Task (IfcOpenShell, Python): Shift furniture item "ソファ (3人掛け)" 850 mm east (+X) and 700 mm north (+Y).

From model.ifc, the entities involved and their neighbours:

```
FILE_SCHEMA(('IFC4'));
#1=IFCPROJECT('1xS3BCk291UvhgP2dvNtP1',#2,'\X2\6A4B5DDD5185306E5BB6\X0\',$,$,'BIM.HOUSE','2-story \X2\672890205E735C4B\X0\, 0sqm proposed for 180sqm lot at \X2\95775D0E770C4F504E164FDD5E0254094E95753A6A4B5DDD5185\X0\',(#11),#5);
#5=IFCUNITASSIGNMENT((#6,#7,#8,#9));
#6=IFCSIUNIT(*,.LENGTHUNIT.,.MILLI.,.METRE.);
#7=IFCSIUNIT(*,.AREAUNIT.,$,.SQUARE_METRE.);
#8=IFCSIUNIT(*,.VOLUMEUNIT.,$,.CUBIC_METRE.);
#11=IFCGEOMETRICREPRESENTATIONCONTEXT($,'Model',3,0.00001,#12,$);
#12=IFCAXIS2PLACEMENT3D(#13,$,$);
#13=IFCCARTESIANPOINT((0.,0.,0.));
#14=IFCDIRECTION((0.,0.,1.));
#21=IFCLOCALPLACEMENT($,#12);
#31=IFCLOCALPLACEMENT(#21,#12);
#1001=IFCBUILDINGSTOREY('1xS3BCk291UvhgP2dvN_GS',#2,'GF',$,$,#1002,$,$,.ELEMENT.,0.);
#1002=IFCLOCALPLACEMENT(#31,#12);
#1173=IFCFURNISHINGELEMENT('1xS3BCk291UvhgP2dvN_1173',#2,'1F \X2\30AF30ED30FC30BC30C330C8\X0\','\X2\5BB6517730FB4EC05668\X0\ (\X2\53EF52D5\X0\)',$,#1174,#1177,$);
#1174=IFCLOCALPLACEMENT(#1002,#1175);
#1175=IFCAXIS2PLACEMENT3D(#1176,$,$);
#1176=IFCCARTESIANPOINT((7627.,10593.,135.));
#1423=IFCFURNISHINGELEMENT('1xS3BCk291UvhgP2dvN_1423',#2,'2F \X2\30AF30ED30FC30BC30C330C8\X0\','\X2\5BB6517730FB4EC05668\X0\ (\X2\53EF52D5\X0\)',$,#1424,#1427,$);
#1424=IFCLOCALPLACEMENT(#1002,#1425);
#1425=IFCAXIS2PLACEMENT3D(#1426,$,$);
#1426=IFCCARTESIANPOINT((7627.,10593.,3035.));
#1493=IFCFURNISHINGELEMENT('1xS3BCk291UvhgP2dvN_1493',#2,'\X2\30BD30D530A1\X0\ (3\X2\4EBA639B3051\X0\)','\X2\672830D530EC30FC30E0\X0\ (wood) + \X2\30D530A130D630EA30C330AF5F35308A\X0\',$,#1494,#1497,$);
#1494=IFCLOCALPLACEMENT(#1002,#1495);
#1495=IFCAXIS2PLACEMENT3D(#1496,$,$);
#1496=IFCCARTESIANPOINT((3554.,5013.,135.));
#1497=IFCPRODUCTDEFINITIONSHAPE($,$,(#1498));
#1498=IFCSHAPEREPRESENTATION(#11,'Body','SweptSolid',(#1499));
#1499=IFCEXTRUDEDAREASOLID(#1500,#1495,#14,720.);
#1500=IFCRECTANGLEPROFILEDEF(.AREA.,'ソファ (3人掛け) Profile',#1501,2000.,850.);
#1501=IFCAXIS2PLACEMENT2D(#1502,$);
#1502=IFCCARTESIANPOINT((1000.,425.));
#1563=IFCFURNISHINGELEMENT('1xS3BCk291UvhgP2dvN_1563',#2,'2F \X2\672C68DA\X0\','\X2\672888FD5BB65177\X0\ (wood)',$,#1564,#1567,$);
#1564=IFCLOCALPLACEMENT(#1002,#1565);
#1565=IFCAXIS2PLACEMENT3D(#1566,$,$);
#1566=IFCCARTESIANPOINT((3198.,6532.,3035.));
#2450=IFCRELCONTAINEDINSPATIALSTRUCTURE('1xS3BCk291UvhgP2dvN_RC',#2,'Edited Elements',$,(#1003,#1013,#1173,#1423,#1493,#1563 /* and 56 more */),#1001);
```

```python
import ifcopenshell
import ifcopenshell.api.geometry
import ifcopenshell.util.placement

model = ifcopenshell.open("model.ifc")

item = model.by_guid("1xS3BCk291UvhgP2dvN_1493")
matrix = ifcopenshell.util.placement.get_local_placement(item.ObjectPlacement)
matrix[0, 3] += 850.0
matrix[1, 3] += 700.0
ifcopenshell.api.geometry.edit_object_placement(model, product=item, matrix=matrix, is_si=False)

print(ifcopenshell.util.placement.get_local_placement(item.ObjectPlacement).round(3) + 0.0)

model.write("model_v2.ifc")
```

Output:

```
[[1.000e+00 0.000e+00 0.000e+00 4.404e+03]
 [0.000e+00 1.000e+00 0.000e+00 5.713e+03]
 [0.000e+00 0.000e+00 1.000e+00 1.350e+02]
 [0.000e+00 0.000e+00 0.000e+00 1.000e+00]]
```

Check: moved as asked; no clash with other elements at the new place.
